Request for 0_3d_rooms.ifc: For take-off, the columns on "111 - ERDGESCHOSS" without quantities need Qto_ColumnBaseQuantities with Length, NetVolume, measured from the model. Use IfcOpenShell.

First a look at what the model holds.

```python
import ifcopenshell
import ifcopenshell.util.element
import ifcopenshell.util.unit

model = ifcopenshell.open("0_3d_rooms.ifc")
print(model.schema)
for unit_type in ("LENGTHUNIT", "AREAUNIT", "VOLUMEUNIT"):
    print(unit_type, ifcopenshell.util.unit.calculate_unit_scale(model, unit_type))
storey = next(s for s in model.by_type("IfcBuildingStorey") if s.Name == "111 - ERDGESCHOSS")
columns = [e for e in ifcopenshell.util.element.get_decomposition(storey) if e.is_a("IfcColumn")]
for e in sorted(columns, key=lambda e: e.id()):
    print(e.id(), e.is_a(), e.Name, list(ifcopenshell.util.element.get_psets(e, qtos_only=True)), sep=" | ")
```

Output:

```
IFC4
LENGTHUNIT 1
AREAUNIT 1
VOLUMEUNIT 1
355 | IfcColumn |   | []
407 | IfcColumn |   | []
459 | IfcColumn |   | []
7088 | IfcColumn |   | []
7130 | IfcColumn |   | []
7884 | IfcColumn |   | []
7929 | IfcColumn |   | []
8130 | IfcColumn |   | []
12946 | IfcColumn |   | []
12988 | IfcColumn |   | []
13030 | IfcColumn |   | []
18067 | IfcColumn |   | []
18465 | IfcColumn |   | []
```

```python
import ifcopenshell
import ifcopenshell.api.pset
import ifcopenshell.geom
import ifcopenshell.util.element
import ifcopenshell.util.shape
import ifcopenshell.util.unit

model = ifcopenshell.open("0_3d_rooms.ifc")
unit_scale = ifcopenshell.util.unit.calculate_unit_scale(model)
volume_scale = ifcopenshell.util.unit.calculate_unit_scale(model, "VOLUMEUNIT")
settings = ifcopenshell.geom.settings()

storey = next(s for s in model.by_type("IfcBuildingStorey") if s.Name == "111 - ERDGESCHOSS")
columns = [e for e in ifcopenshell.util.element.get_decomposition(storey) if e.is_a("IfcColumn")]

for e in sorted(columns, key=lambda e: e.id()):
    if ifcopenshell.util.element.get_psets(e, qtos_only=True, should_inherit=False):
        continue
    # Geometry comes back in metres, in the element's own axes.
    shape = ifcopenshell.geom.create_shape(settings, e)
    values = {
        "Length": ifcopenshell.util.shape.get_z(shape.geometry) / unit_scale,
        "NetVolume": ifcopenshell.util.shape.get_volume(shape.geometry) / volume_scale,
    }
    qto = ifcopenshell.api.pset.add_qto(model, product=e, name="Qto_ColumnBaseQuantities")
    ifcopenshell.api.pset.edit_qto(model, qto=qto, properties=values)
    print(e.id(), {k: round(v, 3) for k, v in values.items()})

model.write("0_3d_rooms_v2.ifc")
```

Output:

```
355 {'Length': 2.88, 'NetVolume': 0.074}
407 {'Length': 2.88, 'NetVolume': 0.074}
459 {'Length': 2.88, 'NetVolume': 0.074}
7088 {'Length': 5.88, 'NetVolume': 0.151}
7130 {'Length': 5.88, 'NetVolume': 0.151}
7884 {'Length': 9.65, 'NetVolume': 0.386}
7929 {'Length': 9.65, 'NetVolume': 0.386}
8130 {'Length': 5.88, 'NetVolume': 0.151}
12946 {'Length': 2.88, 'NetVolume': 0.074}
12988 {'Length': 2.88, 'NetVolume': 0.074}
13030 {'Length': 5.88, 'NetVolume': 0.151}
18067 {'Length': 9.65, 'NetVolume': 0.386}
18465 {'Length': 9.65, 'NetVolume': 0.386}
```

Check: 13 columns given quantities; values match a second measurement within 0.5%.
